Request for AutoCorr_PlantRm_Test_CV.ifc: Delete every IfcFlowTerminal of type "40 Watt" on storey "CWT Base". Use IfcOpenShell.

First a look at what the model holds.

```python
import ifcopenshell
import ifcopenshell.util.element

model = ifcopenshell.open("AutoCorr_PlantRm_Test_CV.ifc")
print(model.schema)
storey = next(s for s in model.by_type("IfcBuildingStorey") if s.Name == "CWT Base")
terminals = [e for e in ifcopenshell.util.element.get_decomposition(storey) if e.is_a("IfcFlowTerminal")]
seen = {}
for e in terminals:
    element_type = ifcopenshell.util.element.get_type(e)
    name = element_type.Name if element_type not in (None, e) else None
    seen[name] = seen.get(name, 0) + 1
for name, count in sorted(seen.items(), key=str):
    print(count, "x", name)
```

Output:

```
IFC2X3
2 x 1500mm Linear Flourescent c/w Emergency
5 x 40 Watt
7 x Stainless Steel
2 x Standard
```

```python
import ifcopenshell
import ifcopenshell.api.root
import ifcopenshell.util.element

model = ifcopenshell.open("AutoCorr_PlantRm_Test_CV.ifc")

storey = next(s for s in model.by_type("IfcBuildingStorey") if s.Name == "CWT Base")
terminals = [e for e in ifcopenshell.util.element.get_decomposition(storey) if e.is_a("IfcFlowTerminal")]
targets = [e for e in terminals if (t := ifcopenshell.util.element.get_type(e)) not in (None, e) and t.Name == "40 Watt"]

for e in targets:
    ifcopenshell.api.root.remove_product(model, product=e)
print(len(targets), "removed")

model.write("AutoCorr_PlantRm_Test_CV_updated.ifc")
```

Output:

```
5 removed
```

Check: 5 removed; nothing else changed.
